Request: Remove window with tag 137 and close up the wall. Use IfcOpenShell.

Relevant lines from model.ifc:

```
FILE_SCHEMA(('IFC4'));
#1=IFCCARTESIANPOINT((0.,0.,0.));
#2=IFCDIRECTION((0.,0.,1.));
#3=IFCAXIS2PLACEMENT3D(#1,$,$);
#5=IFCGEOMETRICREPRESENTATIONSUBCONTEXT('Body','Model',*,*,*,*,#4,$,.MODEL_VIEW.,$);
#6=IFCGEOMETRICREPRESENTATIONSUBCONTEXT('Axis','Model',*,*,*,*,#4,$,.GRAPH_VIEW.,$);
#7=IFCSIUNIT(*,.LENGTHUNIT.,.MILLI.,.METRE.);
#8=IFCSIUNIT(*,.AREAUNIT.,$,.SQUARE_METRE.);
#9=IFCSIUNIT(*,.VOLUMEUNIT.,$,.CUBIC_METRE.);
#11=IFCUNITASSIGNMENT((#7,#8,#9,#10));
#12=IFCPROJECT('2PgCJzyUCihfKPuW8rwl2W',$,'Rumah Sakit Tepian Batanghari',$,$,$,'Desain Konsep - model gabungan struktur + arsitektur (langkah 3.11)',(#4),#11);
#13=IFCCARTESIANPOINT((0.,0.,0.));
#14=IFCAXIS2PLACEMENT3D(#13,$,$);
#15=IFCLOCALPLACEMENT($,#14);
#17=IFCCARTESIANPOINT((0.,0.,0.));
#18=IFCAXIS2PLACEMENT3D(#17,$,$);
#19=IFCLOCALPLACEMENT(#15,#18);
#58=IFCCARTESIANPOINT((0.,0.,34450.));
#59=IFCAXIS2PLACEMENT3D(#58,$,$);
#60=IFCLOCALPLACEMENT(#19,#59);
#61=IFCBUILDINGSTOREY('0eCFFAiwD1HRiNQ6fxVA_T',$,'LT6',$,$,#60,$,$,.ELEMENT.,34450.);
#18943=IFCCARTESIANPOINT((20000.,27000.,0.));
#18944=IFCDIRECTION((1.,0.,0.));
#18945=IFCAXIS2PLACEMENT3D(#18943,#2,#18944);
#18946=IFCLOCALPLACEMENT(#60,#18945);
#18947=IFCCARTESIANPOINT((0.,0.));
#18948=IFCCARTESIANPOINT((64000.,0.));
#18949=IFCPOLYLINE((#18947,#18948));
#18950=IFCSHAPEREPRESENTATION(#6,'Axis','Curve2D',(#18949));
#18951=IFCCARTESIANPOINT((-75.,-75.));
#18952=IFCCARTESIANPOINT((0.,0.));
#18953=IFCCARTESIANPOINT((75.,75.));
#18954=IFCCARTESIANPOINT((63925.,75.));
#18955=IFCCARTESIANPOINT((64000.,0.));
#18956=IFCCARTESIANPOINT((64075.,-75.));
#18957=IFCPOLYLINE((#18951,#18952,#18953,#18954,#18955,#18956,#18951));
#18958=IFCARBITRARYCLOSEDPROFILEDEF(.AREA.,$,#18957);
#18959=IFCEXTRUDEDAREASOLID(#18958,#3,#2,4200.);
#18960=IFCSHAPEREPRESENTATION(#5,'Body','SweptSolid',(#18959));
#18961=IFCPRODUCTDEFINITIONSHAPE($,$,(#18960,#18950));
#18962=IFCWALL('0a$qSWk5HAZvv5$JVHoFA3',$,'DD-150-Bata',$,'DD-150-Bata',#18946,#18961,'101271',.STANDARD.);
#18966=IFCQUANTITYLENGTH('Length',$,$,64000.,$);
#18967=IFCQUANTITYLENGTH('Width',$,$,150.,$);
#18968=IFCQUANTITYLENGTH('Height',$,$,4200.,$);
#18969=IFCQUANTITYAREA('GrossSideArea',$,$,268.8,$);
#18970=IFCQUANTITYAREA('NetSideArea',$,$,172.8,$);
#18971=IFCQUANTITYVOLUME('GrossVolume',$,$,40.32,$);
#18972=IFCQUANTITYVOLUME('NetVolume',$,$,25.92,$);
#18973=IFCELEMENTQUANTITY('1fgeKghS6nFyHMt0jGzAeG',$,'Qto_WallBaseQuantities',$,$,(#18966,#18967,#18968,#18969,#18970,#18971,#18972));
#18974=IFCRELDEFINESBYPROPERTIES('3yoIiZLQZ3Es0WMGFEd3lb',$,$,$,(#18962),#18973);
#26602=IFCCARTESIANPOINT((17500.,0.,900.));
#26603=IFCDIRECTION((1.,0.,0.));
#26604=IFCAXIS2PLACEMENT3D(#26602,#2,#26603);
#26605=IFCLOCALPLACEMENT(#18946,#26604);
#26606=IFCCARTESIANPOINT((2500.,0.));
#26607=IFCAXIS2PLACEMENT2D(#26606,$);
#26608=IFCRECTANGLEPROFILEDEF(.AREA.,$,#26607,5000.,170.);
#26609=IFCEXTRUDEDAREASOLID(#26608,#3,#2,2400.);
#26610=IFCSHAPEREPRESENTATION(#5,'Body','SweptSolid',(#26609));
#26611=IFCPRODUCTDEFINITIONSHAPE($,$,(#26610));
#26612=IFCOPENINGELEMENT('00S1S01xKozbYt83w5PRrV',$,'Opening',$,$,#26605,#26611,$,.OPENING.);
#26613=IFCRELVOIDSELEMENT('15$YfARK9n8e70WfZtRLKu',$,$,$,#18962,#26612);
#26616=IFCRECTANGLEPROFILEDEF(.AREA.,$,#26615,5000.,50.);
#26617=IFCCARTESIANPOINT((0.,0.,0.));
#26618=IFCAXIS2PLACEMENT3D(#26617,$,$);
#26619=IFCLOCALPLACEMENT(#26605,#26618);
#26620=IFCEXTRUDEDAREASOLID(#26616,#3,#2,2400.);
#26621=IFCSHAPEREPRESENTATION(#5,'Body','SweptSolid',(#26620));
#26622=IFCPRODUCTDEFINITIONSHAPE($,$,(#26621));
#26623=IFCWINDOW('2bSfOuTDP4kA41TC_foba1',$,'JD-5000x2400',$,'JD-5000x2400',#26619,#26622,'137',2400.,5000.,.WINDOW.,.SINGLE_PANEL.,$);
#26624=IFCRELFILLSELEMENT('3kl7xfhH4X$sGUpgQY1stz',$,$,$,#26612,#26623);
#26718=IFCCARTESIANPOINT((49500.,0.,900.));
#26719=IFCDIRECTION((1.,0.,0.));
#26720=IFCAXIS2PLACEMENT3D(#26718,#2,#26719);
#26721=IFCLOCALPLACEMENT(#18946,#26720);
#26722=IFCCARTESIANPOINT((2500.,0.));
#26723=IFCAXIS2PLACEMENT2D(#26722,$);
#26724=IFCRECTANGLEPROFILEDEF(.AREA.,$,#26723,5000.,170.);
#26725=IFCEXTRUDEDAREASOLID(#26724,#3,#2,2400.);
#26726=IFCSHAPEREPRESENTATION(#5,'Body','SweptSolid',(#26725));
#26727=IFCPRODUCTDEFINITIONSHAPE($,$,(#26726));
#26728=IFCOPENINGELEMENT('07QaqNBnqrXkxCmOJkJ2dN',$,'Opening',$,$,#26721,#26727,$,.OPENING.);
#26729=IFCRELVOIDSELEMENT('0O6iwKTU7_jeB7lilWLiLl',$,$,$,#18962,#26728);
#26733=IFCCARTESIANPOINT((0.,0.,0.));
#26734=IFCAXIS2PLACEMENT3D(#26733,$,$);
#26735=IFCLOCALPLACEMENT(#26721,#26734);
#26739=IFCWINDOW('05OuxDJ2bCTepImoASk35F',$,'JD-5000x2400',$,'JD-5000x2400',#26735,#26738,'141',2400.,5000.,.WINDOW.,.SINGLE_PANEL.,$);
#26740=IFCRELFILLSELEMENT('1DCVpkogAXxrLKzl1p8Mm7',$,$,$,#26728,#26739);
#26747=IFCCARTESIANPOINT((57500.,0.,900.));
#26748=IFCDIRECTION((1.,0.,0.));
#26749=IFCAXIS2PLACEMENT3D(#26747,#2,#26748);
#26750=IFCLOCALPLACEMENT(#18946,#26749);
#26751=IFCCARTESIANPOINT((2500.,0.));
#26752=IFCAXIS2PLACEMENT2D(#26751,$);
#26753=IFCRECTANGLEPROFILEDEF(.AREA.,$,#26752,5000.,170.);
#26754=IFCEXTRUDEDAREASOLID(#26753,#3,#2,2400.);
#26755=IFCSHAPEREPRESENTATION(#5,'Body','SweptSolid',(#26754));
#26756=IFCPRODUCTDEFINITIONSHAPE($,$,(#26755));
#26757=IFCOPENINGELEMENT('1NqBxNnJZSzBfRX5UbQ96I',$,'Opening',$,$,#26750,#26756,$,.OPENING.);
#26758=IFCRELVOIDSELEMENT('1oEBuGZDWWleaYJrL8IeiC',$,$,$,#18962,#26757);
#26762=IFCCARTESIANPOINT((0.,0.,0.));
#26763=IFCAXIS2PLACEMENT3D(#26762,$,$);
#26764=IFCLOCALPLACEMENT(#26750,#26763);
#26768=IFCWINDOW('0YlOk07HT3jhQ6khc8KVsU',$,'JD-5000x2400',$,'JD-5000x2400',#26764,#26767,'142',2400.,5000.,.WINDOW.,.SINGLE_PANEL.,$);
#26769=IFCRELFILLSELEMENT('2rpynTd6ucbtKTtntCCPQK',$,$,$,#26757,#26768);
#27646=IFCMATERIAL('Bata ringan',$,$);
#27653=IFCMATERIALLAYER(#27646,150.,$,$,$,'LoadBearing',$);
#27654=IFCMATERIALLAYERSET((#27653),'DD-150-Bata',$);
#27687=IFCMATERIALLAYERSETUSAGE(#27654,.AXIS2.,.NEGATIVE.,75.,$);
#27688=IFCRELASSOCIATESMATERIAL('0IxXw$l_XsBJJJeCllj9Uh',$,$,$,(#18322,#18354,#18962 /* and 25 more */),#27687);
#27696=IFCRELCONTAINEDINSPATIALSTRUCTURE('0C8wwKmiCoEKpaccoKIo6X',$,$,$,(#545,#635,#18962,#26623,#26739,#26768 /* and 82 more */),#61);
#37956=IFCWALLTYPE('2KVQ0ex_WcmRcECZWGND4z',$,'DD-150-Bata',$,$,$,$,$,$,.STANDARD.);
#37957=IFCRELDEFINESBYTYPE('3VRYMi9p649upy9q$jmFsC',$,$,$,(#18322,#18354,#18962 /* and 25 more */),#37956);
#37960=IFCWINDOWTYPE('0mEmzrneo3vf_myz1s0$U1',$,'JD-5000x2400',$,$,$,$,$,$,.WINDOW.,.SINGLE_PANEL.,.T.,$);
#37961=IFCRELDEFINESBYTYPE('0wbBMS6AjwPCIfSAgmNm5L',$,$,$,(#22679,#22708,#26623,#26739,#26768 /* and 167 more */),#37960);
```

```python
import ifcopenshell
import ifcopenshell.api.feature
import ifcopenshell.api.pset
import ifcopenshell.api.root
import ifcopenshell.geom
import ifcopenshell.util.element
import ifcopenshell.util.shape
import ifcopenshell.util.unit

model = ifcopenshell.open("model.ifc")
area_scale = ifcopenshell.util.unit.calculate_unit_scale(model, "AREAUNIT")
volume_scale = ifcopenshell.util.unit.calculate_unit_scale(model, "VOLUMEUNIT")
settings = ifcopenshell.geom.settings()


def volume(element):
    """Net volume in cubic metres, openings subtracted."""
    shape = ifcopenshell.geom.create_shape(settings, element)
    return ifcopenshell.util.shape.get_volume(shape.geometry)


window = model.by_guid("2bSfOuTDP4kA41TC_foba1")
opening = window.FillsVoids[0].RelatingOpeningElement
wall = opening.VoidsElements[0].RelatingBuildingElement
before = volume(wall)

ifcopenshell.api.root.remove_product(model, product=window)
ifcopenshell.api.feature.remove_feature(model, feature=opening)

after = volume(wall)
thickness = 0.15  # wall thickness in metres

# Update the wall's stored quantities.
qto = model.by_id(ifcopenshell.util.element.get_pset(wall, "Qto_WallBaseQuantities", should_inherit=False)["id"])
ifcopenshell.api.pset.edit_qto(model, qto=qto, properties={
    "NetSideArea": after / thickness / area_scale,
    "NetVolume": after / volume_scale,
})

print(f"wall volume {before:.3f} -> {after:.3f} m3")

model.write("model_v2.ifc")
```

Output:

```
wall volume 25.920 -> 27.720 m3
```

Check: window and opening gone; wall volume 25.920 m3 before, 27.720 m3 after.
